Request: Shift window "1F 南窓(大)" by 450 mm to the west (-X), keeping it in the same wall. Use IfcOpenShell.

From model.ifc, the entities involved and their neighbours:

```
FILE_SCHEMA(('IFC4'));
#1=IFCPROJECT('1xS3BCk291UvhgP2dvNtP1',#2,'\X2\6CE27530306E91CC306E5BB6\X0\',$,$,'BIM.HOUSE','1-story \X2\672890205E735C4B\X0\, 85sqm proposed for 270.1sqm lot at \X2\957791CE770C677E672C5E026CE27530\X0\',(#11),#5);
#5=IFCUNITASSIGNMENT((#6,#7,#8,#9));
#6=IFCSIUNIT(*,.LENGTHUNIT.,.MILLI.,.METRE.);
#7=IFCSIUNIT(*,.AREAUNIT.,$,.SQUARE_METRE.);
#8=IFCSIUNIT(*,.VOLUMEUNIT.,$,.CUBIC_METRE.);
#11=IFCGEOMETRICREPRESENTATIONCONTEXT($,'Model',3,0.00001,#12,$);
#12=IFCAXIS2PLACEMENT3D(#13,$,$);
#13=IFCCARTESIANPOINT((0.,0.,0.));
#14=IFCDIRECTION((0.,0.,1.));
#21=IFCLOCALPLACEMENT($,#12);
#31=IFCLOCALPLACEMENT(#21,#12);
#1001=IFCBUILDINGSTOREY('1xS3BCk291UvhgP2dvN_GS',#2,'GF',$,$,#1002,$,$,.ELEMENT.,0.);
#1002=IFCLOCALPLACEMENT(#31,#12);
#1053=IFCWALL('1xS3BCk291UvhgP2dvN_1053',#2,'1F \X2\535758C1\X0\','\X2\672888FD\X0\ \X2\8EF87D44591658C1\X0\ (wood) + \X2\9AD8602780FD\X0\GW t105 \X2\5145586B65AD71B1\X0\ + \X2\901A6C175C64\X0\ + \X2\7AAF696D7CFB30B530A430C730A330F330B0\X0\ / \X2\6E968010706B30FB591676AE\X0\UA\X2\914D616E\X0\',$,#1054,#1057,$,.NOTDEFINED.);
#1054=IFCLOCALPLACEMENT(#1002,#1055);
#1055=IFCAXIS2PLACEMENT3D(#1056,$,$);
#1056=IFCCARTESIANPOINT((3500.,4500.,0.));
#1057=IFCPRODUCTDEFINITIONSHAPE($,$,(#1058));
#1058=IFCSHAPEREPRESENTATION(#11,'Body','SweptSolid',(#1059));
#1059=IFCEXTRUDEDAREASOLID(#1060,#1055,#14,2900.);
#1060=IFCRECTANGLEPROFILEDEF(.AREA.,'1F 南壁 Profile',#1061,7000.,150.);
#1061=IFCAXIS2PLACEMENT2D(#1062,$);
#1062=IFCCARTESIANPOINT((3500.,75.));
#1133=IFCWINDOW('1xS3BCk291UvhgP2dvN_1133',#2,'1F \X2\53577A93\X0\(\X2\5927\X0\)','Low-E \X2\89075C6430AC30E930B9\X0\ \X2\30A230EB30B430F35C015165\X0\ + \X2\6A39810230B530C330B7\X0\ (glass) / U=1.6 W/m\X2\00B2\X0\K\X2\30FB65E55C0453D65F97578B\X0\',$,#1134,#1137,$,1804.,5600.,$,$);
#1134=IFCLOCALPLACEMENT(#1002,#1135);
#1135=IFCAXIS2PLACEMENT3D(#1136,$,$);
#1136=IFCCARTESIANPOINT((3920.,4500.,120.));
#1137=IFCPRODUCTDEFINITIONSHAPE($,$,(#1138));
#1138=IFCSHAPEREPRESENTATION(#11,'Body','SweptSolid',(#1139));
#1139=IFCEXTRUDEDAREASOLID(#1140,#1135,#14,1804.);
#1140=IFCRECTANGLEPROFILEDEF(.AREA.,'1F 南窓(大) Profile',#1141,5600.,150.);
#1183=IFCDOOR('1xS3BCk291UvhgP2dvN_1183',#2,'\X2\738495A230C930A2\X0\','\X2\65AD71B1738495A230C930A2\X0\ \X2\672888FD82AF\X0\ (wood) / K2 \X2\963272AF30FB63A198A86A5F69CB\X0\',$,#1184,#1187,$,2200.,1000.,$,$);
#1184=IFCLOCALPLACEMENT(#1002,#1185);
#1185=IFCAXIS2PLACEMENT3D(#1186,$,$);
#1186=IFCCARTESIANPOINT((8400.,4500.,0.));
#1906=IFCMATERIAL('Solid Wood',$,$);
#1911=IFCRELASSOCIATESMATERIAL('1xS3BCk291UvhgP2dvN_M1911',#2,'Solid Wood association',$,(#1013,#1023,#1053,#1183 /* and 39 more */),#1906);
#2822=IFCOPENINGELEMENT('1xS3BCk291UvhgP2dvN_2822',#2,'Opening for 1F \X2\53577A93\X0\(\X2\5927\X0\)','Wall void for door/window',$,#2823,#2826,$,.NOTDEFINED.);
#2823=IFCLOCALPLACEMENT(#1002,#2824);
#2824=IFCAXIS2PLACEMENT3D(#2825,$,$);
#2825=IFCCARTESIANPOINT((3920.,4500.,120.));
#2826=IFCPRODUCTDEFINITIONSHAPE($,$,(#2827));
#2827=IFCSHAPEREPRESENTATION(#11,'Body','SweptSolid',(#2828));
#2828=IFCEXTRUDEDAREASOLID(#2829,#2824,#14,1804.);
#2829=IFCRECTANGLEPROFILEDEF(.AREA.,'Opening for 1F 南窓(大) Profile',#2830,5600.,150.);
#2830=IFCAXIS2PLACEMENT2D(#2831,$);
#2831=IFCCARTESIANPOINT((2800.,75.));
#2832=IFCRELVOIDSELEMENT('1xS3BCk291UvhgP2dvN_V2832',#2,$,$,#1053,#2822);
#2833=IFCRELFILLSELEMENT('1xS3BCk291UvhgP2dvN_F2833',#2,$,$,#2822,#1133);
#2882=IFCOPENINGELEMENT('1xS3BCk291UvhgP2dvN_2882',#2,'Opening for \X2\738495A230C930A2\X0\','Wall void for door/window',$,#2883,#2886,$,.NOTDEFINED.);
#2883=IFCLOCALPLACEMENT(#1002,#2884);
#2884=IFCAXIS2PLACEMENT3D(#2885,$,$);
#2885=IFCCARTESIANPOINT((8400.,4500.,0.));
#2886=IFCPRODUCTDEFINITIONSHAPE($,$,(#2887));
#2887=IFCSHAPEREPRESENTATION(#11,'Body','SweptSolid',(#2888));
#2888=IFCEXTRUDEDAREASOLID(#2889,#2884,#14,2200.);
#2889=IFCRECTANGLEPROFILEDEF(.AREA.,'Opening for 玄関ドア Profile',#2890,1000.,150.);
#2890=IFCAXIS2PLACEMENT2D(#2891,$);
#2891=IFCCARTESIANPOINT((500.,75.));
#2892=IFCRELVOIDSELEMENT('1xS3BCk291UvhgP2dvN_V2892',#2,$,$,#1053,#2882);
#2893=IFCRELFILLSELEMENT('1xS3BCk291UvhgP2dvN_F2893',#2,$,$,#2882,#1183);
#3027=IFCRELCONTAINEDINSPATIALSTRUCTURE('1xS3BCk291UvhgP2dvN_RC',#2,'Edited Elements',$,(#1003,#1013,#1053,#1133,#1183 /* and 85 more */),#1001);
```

```python
import ifcopenshell
import ifcopenshell.api.geometry
import ifcopenshell.util.placement
import ifcopenshell.util.unit

model = ifcopenshell.open("model.ifc")
unit_scale = ifcopenshell.util.unit.calculate_unit_scale(model)

window = model.by_guid("1xS3BCk291UvhgP2dvN_1133")
opening = window.FillsVoids[0].RelatingOpeningElement
wall = opening.VoidsElements[0].RelatingBuildingElement

wall_matrix = ifcopenshell.util.placement.get_local_placement(wall.ObjectPlacement)
shift = wall_matrix[:3, 0] * -0.45 / unit_scale
before = ifcopenshell.util.placement.get_local_placement(window.ObjectPlacement)[:3, 3].copy()

# The window is not placed relative to its opening, so move both.
for product in (opening, window):
    matrix = ifcopenshell.util.placement.get_local_placement(product.ObjectPlacement)
    matrix[:3, 3] += shift
    ifcopenshell.api.geometry.edit_object_placement(model, product=product, matrix=matrix, is_si=False)

after = ifcopenshell.util.placement.get_local_placement(window.ObjectPlacement)[:3, 3]
print("window moved by", (after - before).round(3) + 0.0)

model.write("model_rev.ifc")
```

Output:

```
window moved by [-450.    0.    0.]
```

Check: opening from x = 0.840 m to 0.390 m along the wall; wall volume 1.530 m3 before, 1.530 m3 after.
